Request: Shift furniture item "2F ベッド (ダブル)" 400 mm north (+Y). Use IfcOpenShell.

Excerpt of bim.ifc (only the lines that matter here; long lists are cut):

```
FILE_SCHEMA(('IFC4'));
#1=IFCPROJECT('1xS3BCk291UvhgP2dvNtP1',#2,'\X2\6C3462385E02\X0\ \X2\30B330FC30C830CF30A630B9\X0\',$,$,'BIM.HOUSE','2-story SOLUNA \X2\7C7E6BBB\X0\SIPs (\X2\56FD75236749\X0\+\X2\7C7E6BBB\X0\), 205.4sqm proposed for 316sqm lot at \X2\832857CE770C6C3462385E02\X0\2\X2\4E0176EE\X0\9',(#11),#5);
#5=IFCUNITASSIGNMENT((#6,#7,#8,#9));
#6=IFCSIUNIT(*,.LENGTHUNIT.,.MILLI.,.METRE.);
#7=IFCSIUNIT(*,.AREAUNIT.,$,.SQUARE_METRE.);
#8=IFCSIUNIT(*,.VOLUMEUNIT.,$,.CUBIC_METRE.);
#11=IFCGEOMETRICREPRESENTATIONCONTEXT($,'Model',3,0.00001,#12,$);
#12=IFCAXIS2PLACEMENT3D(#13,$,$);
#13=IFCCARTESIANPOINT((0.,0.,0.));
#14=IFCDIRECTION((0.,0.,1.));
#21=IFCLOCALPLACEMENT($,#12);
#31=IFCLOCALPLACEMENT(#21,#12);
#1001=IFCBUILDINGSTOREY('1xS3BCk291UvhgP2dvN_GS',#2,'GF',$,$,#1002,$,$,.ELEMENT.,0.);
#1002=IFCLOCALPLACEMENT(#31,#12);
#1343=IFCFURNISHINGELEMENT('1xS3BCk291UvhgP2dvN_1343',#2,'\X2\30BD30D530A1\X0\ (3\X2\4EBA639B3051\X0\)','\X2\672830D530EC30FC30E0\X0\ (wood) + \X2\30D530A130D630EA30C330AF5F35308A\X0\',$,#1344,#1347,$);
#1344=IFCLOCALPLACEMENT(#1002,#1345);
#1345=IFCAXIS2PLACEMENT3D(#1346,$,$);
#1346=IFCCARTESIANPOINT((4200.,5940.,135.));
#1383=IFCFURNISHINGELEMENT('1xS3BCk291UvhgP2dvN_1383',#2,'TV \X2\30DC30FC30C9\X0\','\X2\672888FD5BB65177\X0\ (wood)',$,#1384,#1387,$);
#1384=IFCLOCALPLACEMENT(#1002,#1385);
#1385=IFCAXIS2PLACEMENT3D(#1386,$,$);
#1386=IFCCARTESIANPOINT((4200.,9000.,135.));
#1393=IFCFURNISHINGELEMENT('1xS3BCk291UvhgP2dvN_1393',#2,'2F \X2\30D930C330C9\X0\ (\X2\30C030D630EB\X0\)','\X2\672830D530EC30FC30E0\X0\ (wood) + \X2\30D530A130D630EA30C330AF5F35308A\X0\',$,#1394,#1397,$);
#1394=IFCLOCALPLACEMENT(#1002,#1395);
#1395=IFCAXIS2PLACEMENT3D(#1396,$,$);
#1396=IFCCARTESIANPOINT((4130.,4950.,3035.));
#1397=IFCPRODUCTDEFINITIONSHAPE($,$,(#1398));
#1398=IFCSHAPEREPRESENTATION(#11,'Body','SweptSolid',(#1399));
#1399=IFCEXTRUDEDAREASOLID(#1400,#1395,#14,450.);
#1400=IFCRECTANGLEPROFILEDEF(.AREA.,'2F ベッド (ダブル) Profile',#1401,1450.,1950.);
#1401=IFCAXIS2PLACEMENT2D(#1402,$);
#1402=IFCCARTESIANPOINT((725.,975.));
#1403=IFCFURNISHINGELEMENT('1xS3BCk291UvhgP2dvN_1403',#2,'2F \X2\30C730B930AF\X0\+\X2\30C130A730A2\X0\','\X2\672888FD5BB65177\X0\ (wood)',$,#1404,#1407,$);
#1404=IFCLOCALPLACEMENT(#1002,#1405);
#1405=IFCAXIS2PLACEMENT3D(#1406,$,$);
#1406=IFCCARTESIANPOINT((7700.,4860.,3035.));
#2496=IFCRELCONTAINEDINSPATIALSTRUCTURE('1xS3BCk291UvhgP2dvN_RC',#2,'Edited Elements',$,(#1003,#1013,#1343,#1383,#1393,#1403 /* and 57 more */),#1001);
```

```python
import ifcopenshell
import ifcopenshell.api.geometry
import ifcopenshell.util.placement
import ifcopenshell.util.unit

model = ifcopenshell.open("bim.ifc")
unit_scale = ifcopenshell.util.unit.calculate_unit_scale(model)

item = model.by_id(1393)
matrix = ifcopenshell.util.placement.get_local_placement(item.ObjectPlacement)
matrix[1, 3] += 0.4 / unit_scale
ifcopenshell.api.geometry.edit_object_placement(model, product=item, matrix=matrix, is_si=False)

print(ifcopenshell.util.placement.get_local_placement(item.ObjectPlacement).round(3) + 0.0)

model.write("bim-out.ifc")
```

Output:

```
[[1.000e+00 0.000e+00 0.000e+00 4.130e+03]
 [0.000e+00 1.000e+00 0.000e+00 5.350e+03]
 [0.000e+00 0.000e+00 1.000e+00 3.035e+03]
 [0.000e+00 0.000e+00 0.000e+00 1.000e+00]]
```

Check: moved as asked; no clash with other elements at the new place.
